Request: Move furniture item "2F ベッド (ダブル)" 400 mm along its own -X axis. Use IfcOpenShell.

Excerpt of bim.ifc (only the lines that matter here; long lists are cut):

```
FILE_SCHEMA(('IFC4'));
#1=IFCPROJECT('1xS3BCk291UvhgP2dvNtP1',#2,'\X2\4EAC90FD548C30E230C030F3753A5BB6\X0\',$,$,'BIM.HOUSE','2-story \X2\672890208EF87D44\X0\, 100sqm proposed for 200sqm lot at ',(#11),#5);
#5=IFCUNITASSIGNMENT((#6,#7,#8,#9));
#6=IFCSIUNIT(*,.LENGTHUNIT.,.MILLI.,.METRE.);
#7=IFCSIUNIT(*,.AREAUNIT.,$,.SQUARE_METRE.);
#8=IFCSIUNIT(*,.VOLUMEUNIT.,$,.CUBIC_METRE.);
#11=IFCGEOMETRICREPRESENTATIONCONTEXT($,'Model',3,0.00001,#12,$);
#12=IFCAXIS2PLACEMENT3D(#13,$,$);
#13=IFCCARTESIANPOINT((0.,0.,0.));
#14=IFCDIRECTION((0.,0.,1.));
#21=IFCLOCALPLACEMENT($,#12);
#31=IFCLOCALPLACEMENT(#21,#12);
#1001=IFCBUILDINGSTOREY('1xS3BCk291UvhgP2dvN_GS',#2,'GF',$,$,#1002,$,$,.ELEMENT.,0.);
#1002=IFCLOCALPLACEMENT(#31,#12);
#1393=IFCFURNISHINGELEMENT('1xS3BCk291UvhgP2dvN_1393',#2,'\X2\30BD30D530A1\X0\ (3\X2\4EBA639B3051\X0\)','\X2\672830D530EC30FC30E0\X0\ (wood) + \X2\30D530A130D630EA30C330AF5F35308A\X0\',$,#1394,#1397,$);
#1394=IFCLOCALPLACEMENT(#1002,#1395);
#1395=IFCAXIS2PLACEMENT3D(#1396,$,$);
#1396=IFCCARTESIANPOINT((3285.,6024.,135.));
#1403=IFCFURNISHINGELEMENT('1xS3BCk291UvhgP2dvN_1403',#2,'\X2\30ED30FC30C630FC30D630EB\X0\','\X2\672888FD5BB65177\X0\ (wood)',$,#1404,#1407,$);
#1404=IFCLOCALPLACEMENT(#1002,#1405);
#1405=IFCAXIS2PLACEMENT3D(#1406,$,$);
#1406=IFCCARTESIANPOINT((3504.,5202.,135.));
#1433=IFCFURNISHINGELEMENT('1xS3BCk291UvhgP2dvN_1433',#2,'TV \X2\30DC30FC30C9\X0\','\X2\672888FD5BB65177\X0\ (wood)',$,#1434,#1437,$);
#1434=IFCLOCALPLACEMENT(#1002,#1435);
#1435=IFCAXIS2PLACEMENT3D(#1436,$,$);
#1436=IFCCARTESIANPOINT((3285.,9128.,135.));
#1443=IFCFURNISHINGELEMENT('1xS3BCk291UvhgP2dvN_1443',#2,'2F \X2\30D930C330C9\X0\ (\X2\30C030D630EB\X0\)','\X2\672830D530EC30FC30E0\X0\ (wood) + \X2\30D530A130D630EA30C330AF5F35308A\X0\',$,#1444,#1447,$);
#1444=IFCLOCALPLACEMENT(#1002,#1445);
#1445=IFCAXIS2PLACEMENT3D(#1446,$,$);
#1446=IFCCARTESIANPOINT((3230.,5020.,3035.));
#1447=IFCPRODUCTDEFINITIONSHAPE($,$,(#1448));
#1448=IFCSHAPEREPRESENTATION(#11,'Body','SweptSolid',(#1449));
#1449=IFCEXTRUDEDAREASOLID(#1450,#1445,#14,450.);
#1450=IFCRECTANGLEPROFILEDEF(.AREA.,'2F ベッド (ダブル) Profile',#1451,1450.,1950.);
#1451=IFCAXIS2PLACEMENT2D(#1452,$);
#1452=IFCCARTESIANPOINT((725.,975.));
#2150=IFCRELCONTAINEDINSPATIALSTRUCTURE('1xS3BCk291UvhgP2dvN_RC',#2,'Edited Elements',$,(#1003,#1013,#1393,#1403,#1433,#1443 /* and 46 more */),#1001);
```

```python
import ifcopenshell
import ifcopenshell.api.geometry
import ifcopenshell.util.placement

model = ifcopenshell.open("bim.ifc")

item = model.by_guid("1xS3BCk291UvhgP2dvN_1443")
matrix = ifcopenshell.util.placement.get_local_placement(item.ObjectPlacement)
matrix[:3, 3] -= matrix[:3, 0] * 400.0
ifcopenshell.api.geometry.edit_object_placement(model, product=item, matrix=matrix, is_si=False)

print(ifcopenshell.util.placement.get_local_placement(item.ObjectPlacement).round(3) + 0.0)

model.write("bim_v2.ifc")
```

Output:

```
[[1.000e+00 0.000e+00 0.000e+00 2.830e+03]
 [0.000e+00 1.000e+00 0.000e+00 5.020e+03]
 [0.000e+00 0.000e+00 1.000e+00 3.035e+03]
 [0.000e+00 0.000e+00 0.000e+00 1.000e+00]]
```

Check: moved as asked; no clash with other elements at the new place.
